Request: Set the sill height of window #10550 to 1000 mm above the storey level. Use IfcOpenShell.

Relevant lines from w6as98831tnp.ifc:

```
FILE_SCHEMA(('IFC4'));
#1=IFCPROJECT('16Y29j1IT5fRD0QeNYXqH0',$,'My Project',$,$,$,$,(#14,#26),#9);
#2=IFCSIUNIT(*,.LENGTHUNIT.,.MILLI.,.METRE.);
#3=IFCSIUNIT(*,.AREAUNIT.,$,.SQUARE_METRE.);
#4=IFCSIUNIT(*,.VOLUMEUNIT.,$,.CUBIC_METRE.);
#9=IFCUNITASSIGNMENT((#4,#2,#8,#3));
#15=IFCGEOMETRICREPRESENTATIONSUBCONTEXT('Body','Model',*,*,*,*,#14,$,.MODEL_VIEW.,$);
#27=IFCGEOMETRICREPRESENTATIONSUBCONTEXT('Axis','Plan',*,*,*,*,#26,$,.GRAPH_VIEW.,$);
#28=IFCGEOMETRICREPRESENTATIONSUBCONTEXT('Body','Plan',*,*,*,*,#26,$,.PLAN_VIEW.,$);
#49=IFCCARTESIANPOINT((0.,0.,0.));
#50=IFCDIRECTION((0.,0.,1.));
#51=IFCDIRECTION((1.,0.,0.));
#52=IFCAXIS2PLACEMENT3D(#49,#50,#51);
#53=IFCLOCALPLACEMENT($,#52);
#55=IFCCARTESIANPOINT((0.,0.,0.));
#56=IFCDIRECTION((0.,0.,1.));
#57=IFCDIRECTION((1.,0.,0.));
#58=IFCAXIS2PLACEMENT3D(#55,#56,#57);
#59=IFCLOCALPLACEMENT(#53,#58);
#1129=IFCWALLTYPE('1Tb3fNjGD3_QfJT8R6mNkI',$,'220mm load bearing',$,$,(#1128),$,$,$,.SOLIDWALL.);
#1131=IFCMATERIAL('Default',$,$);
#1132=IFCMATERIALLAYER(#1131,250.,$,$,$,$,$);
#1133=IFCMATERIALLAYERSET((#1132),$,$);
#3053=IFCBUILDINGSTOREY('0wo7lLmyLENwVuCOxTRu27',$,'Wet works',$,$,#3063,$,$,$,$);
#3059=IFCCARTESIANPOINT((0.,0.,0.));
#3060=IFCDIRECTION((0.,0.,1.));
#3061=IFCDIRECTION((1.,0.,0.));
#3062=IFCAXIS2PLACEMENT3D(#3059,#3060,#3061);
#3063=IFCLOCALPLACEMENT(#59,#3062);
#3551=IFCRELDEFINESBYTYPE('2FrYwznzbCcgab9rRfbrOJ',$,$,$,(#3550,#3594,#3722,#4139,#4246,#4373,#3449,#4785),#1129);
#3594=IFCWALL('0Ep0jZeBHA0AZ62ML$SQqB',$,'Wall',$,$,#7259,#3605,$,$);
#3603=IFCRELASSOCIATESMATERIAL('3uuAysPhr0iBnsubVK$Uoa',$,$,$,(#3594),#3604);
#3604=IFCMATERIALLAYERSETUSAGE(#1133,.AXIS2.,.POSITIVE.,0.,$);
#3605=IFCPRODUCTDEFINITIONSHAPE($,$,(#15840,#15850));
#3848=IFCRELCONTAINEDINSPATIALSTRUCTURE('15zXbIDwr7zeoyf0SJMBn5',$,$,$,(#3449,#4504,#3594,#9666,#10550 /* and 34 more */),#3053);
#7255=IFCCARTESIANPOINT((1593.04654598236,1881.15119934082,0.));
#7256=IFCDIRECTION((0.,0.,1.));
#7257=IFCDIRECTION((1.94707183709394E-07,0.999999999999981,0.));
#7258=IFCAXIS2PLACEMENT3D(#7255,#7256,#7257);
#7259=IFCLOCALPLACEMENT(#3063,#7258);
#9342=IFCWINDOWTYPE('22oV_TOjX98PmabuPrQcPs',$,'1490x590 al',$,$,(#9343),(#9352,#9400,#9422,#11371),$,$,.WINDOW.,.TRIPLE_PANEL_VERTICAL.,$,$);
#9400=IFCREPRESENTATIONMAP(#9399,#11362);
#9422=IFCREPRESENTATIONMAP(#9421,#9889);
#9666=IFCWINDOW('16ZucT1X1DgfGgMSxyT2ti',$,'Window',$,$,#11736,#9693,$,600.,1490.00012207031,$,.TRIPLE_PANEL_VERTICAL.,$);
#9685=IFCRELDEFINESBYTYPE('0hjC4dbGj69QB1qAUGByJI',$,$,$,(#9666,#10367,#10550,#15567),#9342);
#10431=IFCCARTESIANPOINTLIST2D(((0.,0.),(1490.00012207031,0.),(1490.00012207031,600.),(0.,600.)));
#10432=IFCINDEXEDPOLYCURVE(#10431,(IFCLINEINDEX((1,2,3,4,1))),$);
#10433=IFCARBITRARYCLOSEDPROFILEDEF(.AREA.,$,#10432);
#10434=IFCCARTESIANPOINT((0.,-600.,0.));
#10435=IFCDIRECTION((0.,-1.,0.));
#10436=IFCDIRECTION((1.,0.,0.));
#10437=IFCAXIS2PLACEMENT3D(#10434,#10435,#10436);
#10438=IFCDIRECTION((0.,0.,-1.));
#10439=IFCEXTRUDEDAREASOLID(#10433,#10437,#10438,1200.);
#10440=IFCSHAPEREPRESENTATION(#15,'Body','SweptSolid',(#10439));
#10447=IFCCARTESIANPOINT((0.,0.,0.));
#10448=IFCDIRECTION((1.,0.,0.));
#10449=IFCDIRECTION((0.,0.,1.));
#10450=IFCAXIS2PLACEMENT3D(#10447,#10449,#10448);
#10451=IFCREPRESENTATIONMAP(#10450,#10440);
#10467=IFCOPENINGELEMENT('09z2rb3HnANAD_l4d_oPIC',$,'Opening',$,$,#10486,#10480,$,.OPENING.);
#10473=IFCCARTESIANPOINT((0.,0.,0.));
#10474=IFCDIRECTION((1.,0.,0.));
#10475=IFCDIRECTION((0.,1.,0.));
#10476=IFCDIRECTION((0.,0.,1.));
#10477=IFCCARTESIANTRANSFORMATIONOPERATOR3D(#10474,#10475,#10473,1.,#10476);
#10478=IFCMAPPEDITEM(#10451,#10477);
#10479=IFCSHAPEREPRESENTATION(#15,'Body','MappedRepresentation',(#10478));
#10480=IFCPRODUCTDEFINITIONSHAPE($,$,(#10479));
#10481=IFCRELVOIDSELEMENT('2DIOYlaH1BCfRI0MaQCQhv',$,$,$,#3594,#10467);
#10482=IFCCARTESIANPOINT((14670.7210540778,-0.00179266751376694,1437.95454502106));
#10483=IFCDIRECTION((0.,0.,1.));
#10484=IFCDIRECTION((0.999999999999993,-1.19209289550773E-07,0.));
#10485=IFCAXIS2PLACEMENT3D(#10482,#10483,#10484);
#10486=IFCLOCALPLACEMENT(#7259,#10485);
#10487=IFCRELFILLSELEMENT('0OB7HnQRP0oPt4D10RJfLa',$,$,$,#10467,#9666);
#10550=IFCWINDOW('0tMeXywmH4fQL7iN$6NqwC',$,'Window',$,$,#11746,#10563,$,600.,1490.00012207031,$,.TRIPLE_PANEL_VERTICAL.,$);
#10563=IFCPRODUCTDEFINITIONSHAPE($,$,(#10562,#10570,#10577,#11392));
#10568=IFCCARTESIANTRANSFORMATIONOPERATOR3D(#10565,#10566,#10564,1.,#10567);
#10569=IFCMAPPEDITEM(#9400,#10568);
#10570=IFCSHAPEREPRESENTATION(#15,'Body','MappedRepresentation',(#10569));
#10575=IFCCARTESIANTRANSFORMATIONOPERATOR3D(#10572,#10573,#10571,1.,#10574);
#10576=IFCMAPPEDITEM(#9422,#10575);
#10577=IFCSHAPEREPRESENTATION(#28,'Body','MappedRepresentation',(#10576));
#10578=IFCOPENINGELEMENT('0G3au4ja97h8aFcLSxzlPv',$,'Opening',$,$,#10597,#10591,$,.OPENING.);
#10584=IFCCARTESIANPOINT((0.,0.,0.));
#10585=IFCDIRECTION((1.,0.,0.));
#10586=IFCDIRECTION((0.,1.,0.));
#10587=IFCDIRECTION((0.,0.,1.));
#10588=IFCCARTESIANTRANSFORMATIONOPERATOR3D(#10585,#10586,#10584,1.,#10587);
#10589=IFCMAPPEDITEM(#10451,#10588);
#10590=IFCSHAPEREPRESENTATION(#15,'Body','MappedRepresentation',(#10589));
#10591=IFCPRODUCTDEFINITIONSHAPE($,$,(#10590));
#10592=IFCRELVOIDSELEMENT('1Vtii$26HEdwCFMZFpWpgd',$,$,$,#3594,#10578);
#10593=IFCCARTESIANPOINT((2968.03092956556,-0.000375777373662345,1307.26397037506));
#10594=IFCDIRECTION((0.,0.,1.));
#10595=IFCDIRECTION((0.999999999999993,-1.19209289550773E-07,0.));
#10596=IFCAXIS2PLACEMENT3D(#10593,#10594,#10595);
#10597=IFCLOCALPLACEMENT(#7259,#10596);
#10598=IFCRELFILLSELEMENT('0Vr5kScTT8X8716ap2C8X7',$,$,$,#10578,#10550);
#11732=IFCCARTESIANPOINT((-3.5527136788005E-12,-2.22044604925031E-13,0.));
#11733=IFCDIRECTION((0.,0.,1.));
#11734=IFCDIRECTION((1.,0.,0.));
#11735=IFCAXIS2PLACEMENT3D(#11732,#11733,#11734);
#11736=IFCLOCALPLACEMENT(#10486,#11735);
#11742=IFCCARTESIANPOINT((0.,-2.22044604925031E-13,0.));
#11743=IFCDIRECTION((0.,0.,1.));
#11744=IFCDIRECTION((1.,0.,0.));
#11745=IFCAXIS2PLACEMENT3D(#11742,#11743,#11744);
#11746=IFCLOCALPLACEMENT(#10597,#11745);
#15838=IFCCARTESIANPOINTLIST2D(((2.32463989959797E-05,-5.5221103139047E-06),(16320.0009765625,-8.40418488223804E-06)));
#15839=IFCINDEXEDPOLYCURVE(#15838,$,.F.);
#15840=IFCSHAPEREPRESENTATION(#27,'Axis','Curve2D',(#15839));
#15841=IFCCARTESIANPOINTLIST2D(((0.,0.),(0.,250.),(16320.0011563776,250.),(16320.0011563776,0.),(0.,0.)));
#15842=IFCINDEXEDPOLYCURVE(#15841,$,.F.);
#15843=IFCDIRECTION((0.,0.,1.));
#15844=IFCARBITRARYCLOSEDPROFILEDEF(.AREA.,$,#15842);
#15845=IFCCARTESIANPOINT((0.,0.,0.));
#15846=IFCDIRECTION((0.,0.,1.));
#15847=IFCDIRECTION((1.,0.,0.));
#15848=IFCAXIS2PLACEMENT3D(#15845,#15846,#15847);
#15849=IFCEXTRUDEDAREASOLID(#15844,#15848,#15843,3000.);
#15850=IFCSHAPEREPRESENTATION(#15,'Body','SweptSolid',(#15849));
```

```python
import numpy as np
import ifcopenshell
import ifcopenshell.api.geometry
import ifcopenshell.geom
import ifcopenshell.util.element
import ifcopenshell.util.placement
import ifcopenshell.util.shape
import ifcopenshell.util.unit

model = ifcopenshell.open("w6as98831tnp.ifc")
unit_scale = ifcopenshell.util.unit.calculate_unit_scale(model)

window = model.by_id(10550)
opening = window.FillsVoids[0].RelatingOpeningElement
storey = ifcopenshell.util.element.get_container(window, ifc_class="IfcBuildingStorey")
level = ifcopenshell.util.placement.get_local_placement(storey.ObjectPlacement)[2, 3]

# The opening's origin need not be at the sill, so measure its lowest point.
shape = ifcopenshell.geom.create_shape(ifcopenshell.geom.settings(), opening)
bottom = ifcopenshell.util.shape.get_shape_bottom_elevation(shape, shape.geometry) / unit_scale
dz = level + 1000.0 - bottom

shift = np.array([0.0, 0.0, dz])
# The window is placed relative to its opening, so it follows when the opening moves.
matrix = ifcopenshell.util.placement.get_local_placement(opening.ObjectPlacement)
matrix[:3, 3] += shift
ifcopenshell.api.geometry.edit_object_placement(
    model, product=opening, matrix=matrix, is_si=False, should_transform_children=True
)

print(f"moved by {dz * unit_scale:+.3f} m")

model.write("w6as98831tnp_v2.ifc")
```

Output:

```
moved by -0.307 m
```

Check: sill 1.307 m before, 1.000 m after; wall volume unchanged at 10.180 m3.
